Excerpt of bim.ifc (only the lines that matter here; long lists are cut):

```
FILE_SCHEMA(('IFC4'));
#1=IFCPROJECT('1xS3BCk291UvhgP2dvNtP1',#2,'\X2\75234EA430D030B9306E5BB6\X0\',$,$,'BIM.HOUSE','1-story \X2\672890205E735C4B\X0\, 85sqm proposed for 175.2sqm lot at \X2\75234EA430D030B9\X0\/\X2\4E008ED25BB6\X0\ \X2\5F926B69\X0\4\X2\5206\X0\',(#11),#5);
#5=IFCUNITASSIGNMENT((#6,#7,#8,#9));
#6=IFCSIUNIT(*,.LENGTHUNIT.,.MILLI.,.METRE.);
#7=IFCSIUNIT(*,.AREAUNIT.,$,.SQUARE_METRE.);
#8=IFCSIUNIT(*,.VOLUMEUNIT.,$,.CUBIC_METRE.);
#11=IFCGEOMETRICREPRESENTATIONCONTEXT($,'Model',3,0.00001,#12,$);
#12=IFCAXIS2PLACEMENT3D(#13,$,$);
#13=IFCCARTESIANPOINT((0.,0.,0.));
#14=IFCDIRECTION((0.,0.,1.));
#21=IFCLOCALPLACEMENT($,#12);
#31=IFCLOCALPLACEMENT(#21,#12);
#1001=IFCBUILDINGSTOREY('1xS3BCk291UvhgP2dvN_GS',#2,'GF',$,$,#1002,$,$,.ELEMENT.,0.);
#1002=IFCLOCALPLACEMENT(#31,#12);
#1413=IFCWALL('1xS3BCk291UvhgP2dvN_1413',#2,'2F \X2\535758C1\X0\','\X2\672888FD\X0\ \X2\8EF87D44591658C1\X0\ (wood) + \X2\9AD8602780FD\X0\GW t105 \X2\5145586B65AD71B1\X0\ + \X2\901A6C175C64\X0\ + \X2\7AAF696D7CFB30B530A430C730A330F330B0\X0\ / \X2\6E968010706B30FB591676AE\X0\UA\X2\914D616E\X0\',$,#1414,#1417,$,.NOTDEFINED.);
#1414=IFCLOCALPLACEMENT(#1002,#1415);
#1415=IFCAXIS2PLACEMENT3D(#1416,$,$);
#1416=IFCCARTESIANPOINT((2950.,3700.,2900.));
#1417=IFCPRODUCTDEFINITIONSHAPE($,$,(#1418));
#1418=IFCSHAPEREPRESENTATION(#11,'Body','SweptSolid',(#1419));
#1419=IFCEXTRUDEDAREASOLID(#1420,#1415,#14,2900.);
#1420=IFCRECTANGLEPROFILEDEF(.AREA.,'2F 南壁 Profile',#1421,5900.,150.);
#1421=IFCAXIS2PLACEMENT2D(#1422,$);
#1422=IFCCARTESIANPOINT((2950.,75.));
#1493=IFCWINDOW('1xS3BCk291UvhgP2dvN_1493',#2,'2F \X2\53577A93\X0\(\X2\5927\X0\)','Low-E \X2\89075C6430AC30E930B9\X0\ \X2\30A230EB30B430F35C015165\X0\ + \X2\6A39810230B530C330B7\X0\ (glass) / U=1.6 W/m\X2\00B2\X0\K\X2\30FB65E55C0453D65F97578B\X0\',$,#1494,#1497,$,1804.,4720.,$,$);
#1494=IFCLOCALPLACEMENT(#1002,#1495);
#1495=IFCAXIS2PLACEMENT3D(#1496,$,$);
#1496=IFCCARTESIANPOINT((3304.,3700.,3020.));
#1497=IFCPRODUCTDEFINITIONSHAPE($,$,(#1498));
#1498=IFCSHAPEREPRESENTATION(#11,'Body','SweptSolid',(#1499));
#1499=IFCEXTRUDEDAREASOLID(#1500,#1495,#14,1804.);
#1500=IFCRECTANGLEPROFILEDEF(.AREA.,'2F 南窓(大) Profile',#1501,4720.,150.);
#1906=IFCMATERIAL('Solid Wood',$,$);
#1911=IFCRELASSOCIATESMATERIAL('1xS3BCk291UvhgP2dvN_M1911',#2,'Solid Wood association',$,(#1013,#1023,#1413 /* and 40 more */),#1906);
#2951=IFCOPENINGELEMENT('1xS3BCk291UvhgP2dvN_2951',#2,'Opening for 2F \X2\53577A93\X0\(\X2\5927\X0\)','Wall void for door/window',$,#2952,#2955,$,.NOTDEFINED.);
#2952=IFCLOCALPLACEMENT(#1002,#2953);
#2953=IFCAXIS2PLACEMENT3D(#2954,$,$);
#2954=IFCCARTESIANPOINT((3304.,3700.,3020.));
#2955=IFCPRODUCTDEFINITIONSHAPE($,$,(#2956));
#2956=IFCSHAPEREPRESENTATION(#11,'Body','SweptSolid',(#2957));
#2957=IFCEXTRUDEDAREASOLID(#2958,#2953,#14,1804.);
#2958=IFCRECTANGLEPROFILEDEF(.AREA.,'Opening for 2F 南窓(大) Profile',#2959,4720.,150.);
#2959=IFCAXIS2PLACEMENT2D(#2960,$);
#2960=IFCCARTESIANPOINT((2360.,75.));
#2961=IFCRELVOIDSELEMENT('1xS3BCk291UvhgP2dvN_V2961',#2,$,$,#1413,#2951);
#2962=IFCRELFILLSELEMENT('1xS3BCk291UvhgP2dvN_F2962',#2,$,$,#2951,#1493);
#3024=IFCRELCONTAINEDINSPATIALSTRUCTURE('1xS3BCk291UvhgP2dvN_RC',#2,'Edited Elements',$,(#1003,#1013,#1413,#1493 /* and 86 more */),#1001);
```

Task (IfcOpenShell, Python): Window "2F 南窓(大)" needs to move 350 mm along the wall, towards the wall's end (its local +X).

```python
import ifcopenshell
import ifcopenshell.api.geometry
import ifcopenshell.util.placement
import ifcopenshell.util.unit

model = ifcopenshell.open("bim.ifc")
unit_scale = ifcopenshell.util.unit.calculate_unit_scale(model)

window = model.by_guid("1xS3BCk291UvhgP2dvN_1493")
opening = window.FillsVoids[0].RelatingOpeningElement
wall = opening.VoidsElements[0].RelatingBuildingElement

wall_matrix = ifcopenshell.util.placement.get_local_placement(wall.ObjectPlacement)
shift = wall_matrix[:3, 0] * 0.35 / unit_scale
before = ifcopenshell.util.placement.get_local_placement(window.ObjectPlacement)[:3, 3].copy()

# The window is not placed relative to its opening, so move both.
for product in (opening, window):
    matrix = ifcopenshell.util.placement.get_local_placement(product.ObjectPlacement)
    matrix[:3, 3] += shift
    ifcopenshell.api.geometry.edit_object_placement(model, product=product, matrix=matrix, is_si=False)

after = ifcopenshell.util.placement.get_local_placement(window.ObjectPlacement)[:3, 3]
print("window moved by", (after - before).round(3) + 0.0)

model.write("bim-out.ifc")
```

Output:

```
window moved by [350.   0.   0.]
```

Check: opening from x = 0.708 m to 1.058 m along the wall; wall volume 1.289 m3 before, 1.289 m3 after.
